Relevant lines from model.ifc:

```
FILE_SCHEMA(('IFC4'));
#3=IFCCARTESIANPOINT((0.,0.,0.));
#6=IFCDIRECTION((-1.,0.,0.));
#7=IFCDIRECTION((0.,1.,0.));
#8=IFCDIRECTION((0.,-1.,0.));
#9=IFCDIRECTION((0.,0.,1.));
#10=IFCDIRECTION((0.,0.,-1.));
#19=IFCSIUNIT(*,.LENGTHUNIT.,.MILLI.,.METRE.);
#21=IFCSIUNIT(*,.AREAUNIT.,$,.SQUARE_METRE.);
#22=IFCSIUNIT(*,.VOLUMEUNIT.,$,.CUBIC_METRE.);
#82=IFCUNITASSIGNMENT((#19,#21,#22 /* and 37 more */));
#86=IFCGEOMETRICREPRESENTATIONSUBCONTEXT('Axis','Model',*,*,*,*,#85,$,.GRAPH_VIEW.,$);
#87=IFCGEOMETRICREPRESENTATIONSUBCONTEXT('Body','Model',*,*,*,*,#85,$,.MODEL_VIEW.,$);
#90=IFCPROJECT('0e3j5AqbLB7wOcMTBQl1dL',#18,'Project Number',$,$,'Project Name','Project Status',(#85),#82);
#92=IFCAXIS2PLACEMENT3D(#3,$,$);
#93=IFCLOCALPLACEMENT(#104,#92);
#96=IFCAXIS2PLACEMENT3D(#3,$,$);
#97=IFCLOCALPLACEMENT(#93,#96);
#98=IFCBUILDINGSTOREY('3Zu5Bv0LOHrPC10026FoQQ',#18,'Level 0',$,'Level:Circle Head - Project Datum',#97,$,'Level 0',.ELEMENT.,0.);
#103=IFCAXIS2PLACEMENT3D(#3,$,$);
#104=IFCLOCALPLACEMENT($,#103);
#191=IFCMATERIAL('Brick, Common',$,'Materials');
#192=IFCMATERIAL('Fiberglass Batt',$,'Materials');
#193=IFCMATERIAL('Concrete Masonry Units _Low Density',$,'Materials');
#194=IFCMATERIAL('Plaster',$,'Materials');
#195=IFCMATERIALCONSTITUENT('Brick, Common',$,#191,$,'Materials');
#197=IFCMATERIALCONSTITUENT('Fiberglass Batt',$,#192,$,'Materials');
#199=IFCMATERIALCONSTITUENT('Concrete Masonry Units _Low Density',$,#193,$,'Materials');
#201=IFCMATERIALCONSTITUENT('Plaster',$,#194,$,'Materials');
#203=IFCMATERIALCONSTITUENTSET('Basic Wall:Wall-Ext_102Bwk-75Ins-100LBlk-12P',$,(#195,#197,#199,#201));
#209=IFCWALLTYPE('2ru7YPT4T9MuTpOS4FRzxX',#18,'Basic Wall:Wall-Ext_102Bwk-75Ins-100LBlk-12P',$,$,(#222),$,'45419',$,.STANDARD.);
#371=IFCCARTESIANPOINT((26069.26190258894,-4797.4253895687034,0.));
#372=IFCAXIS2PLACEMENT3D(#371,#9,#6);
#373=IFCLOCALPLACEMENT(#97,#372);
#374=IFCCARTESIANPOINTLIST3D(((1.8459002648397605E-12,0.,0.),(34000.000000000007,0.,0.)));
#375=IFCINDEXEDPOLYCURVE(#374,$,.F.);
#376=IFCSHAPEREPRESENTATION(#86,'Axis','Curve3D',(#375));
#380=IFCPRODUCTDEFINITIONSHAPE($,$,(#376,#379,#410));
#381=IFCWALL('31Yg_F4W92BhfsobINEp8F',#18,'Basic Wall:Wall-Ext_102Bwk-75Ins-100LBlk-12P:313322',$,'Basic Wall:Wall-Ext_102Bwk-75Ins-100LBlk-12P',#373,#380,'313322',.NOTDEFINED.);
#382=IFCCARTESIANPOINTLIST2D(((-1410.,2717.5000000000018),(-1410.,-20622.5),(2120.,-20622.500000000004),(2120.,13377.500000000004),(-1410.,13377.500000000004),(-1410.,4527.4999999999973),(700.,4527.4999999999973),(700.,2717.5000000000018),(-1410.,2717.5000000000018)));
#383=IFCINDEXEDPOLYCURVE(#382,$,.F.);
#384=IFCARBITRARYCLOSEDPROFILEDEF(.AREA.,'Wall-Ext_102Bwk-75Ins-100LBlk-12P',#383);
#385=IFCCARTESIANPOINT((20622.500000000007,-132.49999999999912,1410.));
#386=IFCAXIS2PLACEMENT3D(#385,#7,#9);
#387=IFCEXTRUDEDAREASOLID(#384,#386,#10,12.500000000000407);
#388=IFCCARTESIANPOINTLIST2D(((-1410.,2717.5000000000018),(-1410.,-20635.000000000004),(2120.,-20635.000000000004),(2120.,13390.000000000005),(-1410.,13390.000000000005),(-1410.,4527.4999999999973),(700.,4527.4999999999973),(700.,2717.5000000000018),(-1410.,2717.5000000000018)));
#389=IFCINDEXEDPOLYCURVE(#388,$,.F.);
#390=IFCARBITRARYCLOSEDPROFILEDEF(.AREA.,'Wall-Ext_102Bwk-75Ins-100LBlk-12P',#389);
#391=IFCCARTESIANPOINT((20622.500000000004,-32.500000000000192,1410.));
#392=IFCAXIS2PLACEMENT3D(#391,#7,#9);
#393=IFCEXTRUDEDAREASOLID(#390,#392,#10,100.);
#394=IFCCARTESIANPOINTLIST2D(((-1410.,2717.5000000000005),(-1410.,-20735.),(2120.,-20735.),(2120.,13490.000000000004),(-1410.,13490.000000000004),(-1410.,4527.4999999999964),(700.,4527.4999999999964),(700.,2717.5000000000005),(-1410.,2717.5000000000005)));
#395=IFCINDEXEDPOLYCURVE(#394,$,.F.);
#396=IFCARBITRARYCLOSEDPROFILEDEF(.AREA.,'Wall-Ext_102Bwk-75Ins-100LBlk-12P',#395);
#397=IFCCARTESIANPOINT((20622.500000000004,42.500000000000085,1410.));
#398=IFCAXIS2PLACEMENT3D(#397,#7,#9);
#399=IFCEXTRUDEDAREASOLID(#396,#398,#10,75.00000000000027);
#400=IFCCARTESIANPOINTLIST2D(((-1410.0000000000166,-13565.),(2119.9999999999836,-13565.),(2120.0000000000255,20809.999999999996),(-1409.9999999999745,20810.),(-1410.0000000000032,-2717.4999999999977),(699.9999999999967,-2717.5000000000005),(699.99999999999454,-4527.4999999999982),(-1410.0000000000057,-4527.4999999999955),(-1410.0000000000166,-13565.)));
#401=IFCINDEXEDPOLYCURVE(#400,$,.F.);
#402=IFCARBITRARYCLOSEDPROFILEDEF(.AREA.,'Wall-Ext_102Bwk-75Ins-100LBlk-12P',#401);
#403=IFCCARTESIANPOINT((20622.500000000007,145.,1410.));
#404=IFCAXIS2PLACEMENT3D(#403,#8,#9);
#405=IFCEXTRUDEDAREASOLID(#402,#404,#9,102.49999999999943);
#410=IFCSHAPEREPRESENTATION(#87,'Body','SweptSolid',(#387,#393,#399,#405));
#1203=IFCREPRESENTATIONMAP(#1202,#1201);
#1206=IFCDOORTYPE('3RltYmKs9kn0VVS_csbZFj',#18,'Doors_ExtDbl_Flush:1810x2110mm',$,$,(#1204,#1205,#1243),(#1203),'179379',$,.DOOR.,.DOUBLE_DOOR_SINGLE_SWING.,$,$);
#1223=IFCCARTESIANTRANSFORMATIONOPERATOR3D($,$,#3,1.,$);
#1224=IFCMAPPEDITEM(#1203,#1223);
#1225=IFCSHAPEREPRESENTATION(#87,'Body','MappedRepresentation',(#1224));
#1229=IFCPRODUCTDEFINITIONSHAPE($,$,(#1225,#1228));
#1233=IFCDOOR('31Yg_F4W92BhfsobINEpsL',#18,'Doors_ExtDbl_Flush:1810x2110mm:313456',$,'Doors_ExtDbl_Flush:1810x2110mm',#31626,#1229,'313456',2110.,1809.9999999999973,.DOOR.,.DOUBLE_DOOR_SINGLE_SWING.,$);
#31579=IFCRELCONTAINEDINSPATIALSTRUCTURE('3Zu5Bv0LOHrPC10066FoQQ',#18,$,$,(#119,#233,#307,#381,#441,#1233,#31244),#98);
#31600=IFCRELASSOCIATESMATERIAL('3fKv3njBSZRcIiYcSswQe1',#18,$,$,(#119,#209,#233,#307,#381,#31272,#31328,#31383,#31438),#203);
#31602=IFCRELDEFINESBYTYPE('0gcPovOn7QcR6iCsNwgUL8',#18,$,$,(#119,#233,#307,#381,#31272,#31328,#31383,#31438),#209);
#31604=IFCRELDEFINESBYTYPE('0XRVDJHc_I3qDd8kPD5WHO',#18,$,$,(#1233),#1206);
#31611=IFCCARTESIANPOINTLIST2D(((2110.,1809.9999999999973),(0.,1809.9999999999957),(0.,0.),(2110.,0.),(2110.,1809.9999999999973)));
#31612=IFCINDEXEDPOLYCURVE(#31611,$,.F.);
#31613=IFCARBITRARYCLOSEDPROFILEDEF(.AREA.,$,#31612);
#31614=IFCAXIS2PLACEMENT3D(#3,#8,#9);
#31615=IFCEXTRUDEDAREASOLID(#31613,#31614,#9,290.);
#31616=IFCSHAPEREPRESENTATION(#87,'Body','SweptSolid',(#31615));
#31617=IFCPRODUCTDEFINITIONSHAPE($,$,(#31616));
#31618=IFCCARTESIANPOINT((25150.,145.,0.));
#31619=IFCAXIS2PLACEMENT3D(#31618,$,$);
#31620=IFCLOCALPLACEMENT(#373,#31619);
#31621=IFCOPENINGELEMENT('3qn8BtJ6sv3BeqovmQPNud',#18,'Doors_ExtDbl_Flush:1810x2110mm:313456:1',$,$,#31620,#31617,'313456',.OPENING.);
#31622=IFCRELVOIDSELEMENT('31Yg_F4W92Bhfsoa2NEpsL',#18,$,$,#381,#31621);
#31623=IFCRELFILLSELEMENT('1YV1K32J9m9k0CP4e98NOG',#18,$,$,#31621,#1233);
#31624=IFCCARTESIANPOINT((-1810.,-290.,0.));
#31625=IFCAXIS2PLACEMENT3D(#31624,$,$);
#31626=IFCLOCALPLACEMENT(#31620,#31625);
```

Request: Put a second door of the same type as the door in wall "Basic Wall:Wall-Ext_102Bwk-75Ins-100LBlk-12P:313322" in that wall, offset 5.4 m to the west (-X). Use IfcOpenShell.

```python
import ifcopenshell
import ifcopenshell.api.feature
import ifcopenshell.api.geometry
import ifcopenshell.api.root
import ifcopenshell.geom
import ifcopenshell.util.element
import ifcopenshell.util.placement
import ifcopenshell.util.shape
import ifcopenshell.util.unit

model = ifcopenshell.open("model.ifc")
unit_scale = ifcopenshell.util.unit.calculate_unit_scale(model)
settings = ifcopenshell.geom.settings()


def volume(element):
    """Net volume in cubic metres, openings subtracted."""
    shape = ifcopenshell.geom.create_shape(settings, element)
    return ifcopenshell.util.shape.get_volume(shape.geometry)


def reuse_history(source, copy):
    """copy_class also copies each property set's owner history, people and application; keep the originals."""
    for rel in copy.IsDefinedBy:
        if rel.is_a("IfcRelDefinesByProperties") and (history := rel.RelatingPropertyDefinition.OwnerHistory):
            rel.RelatingPropertyDefinition.OwnerHistory = source.OwnerHistory
            ifcopenshell.util.element.remove_deep2(model, history)


door = model.by_guid("31Yg_F4W92BhfsobINEpsL")
opening = door.FillsVoids[0].RelatingOpeningElement
wall = opening.VoidsElements[0].RelatingBuildingElement
before = volume(wall)
shift = ifcopenshell.util.placement.get_local_placement(wall.ObjectPlacement)[:3, 0] * 5.4 / unit_scale

# copy_class copies the void relationship, type, container and properties, but no geometry.
new_opening = ifcopenshell.api.root.copy_class(model, product=opening)
new_opening.Representation = ifcopenshell.util.element.copy_deep(
    model, opening.Representation, exclude=["IfcGeometricRepresentationContext", "IfcRepresentationMap"]
)
new_opening.Name = "Doors_ExtDbl_Flush:1810x2110mm"
new_opening.Tag = None
new_door = ifcopenshell.api.root.copy_class(model, product=door)
new_door.Representation = ifcopenshell.util.element.copy_deep(
    model, door.Representation, exclude=["IfcGeometricRepresentationContext", "IfcRepresentationMap"]
)
new_door.Name = "Doors_ExtDbl_Flush:1810x2110mm"
new_door.Tag = None
reuse_history(door, new_door)
ifcopenshell.api.feature.add_filling(model, opening=new_opening, element=new_door)

for old, new in ((opening, new_opening), (door, new_door)):
    matrix = ifcopenshell.util.placement.get_local_placement(old.ObjectPlacement)
    matrix[:3, 3] += shift
    ifcopenshell.api.geometry.edit_object_placement(model, product=new, matrix=matrix, is_si=False)

after = volume(wall)

print(f"wall volume {before:.3f} -> {after:.3f} m3")

model.write("model_edited.ifc")
```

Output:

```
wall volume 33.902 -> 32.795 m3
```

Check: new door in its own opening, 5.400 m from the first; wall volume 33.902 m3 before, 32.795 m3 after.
